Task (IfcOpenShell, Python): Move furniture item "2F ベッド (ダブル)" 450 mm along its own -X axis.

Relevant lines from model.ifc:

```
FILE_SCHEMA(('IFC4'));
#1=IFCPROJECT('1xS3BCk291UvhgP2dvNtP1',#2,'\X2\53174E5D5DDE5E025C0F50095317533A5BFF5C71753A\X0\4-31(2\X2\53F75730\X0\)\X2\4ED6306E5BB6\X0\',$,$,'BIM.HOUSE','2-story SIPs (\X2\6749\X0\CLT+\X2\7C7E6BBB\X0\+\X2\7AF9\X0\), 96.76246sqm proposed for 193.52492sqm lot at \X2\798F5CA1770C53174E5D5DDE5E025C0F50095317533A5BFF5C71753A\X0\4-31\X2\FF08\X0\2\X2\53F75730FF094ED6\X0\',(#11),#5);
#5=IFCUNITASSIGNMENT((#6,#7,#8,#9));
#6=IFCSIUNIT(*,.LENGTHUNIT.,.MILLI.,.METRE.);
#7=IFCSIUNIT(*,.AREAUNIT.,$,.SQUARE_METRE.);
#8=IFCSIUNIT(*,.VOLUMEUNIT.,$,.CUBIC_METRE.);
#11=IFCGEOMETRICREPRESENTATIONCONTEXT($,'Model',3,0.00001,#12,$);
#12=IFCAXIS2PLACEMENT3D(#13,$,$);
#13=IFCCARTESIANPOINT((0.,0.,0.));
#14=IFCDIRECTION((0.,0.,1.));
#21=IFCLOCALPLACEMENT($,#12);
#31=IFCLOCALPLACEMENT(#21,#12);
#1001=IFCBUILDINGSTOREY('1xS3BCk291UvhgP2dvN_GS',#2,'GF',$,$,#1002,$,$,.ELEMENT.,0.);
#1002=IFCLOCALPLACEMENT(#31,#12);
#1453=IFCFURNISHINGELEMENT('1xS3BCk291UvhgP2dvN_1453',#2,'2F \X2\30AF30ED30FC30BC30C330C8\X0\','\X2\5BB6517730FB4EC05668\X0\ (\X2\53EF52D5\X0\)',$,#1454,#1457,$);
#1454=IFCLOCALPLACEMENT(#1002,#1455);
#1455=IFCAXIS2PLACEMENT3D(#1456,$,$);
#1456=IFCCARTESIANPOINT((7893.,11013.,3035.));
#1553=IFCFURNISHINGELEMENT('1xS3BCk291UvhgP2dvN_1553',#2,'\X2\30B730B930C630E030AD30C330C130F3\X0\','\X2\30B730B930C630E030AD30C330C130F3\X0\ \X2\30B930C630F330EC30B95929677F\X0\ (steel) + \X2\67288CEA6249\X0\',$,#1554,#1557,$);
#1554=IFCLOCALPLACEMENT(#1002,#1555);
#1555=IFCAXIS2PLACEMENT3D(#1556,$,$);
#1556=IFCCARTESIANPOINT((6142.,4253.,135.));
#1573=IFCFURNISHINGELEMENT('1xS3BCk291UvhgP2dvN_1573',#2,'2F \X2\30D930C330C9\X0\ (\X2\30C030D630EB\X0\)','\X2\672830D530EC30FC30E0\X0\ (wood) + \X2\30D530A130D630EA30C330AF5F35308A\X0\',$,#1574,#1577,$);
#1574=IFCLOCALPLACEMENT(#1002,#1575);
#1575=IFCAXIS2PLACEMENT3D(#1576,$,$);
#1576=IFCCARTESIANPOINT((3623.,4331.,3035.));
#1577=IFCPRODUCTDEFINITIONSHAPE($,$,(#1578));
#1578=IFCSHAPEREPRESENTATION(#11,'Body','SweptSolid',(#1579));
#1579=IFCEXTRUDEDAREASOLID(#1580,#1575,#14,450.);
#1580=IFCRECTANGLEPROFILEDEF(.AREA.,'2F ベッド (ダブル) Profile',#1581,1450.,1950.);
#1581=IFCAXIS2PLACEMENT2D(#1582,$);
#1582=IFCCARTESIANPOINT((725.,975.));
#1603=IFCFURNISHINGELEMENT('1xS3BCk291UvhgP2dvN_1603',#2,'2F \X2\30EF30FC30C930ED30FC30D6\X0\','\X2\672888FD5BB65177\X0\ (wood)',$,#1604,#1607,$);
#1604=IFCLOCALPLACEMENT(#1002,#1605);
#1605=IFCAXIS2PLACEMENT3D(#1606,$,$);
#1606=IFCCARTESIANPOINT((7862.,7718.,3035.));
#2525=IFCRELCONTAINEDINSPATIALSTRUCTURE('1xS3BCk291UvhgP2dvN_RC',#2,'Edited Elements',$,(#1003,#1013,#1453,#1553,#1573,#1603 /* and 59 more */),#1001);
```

```python
import ifcopenshell
import ifcopenshell.api.geometry
import ifcopenshell.util.placement
import ifcopenshell.util.unit

model = ifcopenshell.open("model.ifc")
unit_scale = ifcopenshell.util.unit.calculate_unit_scale(model)

item = model.by_guid("1xS3BCk291UvhgP2dvN_1573")
matrix = ifcopenshell.util.placement.get_local_placement(item.ObjectPlacement)
matrix[:3, 3] -= matrix[:3, 0] * 0.45 / unit_scale
ifcopenshell.api.geometry.edit_object_placement(model, product=item, matrix=matrix, is_si=False)

print(ifcopenshell.util.placement.get_local_placement(item.ObjectPlacement).round(3) + 0.0)

model.write("model_v2.ifc")
```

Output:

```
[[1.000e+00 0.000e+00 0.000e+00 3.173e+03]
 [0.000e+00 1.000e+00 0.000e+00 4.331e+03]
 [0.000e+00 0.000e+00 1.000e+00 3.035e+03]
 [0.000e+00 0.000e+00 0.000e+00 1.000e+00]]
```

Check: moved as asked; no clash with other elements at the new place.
